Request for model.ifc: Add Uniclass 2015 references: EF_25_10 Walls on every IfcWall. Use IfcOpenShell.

First a look at what the model holds.

```python
import ifcopenshell

model = ifcopenshell.open("model.ifc")
print(model.schema)
print("classifications:", [c.Name for c in model.by_type("IfcClassification")])
for ifc_class in ("IfcDoor", "IfcRoof", "IfcStair", "IfcWall", "IfcWindow"):
    print(ifc_class, len(model.by_type(ifc_class)))
```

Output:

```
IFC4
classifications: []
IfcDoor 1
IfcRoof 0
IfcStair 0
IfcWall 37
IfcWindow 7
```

```python
import ifcopenshell
import ifcopenshell.api.classification

model = ifcopenshell.open("model.ifc")

system = ifcopenshell.api.classification.add_classification(model, classification="Uniclass 2015")

codes = {
    "IfcWall": ("EF_25_10", "Walls"),
}
for ifc_class, (code, name) in codes.items():
    products = model.by_type(ifc_class)
    ifcopenshell.api.classification.add_reference(
        model, products=products, classification=system, identification=code, name=name
    )
    print(code, len(products))

model.write("model-out.ifc")
```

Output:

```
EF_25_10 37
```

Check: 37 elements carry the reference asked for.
